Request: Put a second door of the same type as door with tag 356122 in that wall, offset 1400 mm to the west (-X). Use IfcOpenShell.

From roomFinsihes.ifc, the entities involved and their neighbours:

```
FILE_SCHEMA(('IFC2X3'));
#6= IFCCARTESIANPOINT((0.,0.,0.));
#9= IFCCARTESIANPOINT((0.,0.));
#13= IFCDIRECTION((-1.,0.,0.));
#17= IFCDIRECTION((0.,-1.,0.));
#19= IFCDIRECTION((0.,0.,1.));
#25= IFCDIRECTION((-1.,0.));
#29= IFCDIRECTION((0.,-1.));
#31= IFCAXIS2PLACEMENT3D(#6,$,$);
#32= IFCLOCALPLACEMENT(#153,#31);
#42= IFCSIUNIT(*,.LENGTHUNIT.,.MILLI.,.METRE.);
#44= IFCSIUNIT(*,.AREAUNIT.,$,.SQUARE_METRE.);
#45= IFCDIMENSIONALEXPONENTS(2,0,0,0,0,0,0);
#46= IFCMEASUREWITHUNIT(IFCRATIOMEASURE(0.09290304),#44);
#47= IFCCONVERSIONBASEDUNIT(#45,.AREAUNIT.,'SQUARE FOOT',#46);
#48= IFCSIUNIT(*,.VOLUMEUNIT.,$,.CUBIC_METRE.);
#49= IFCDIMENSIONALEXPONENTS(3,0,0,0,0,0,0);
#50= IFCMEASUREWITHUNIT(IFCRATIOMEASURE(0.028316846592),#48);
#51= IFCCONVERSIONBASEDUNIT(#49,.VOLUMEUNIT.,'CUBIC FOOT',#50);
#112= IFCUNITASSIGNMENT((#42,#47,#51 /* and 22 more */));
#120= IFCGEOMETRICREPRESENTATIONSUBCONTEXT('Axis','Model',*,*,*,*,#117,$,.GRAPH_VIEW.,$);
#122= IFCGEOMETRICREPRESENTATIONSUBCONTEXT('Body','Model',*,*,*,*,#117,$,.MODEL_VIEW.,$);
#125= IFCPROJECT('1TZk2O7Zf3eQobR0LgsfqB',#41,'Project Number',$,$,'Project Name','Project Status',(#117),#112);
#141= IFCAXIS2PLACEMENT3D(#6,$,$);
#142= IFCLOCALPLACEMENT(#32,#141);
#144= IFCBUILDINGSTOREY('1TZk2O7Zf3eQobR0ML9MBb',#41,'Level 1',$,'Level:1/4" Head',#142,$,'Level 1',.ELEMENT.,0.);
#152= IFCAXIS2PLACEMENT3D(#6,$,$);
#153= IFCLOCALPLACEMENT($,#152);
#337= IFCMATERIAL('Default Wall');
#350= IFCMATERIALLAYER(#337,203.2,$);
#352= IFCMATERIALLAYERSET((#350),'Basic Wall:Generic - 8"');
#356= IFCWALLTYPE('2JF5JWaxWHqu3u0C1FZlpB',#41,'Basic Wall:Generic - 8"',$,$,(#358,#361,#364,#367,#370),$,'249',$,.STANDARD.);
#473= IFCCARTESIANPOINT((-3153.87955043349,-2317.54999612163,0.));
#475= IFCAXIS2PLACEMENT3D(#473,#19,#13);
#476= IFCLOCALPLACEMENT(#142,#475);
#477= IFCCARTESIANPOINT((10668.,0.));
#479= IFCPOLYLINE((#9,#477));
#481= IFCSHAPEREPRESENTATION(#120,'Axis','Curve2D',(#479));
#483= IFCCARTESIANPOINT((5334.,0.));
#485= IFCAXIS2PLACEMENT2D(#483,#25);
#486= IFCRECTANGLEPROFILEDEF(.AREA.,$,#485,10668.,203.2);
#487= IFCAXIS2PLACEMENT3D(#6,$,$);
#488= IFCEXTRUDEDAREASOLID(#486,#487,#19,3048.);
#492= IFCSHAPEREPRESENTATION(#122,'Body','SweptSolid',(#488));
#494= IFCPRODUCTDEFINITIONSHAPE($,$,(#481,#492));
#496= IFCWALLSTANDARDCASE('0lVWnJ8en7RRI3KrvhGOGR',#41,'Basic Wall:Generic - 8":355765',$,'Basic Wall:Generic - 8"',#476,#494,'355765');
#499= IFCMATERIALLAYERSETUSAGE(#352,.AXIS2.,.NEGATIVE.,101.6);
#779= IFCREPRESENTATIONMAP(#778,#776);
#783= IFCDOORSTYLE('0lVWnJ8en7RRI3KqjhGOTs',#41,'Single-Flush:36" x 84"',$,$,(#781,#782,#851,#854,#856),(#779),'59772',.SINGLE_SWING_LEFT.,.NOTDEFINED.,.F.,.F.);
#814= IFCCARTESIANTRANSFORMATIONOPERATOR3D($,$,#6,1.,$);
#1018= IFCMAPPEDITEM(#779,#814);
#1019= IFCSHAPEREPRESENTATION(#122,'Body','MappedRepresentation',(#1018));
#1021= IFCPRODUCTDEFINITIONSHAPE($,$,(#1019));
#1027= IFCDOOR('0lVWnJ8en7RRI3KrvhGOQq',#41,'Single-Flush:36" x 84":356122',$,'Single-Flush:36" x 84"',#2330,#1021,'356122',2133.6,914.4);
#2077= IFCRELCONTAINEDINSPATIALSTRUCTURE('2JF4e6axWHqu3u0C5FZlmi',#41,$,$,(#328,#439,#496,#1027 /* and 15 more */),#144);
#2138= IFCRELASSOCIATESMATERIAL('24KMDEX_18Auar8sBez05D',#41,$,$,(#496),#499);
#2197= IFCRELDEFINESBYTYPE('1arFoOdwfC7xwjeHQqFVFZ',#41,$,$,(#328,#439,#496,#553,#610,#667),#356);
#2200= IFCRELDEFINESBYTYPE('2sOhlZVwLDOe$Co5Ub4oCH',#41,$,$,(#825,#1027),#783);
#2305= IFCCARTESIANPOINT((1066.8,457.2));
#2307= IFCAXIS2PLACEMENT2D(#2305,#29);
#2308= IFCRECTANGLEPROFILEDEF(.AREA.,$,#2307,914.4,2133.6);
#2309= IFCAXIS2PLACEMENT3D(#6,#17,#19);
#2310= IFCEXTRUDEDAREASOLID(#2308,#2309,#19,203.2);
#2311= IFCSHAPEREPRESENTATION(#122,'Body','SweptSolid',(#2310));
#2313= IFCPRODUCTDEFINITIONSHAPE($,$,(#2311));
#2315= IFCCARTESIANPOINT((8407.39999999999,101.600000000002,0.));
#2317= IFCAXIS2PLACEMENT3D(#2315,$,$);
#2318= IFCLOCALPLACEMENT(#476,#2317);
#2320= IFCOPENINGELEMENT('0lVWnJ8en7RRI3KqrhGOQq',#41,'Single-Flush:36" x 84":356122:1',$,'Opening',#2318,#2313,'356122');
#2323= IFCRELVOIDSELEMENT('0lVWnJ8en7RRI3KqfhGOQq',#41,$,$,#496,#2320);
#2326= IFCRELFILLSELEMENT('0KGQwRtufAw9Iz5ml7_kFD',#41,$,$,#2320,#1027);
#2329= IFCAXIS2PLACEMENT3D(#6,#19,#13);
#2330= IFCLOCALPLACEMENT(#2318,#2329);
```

```python
import ifcopenshell
import ifcopenshell.api.feature
import ifcopenshell.api.geometry
import ifcopenshell.api.root
import ifcopenshell.geom
import ifcopenshell.util.element
import ifcopenshell.util.placement
import ifcopenshell.util.shape
import ifcopenshell.util.unit

model = ifcopenshell.open("roomFinsihes.ifc")
unit_scale = ifcopenshell.util.unit.calculate_unit_scale(model)
settings = ifcopenshell.geom.settings()


def volume(element):
    """Net volume in cubic metres, openings subtracted."""
    shape = ifcopenshell.geom.create_shape(settings, element)
    return ifcopenshell.util.shape.get_volume(shape.geometry)


def reuse_history(source, copy):
    """copy_class also copies each property set's owner history, people and application; keep the originals."""
    for rel in copy.IsDefinedBy:
        if rel.is_a("IfcRelDefinesByProperties") and (history := rel.RelatingPropertyDefinition.OwnerHistory):
            rel.RelatingPropertyDefinition.OwnerHistory = source.OwnerHistory
            ifcopenshell.util.element.remove_deep2(model, history)


door = model.by_guid("0lVWnJ8en7RRI3KrvhGOQq")
opening = door.FillsVoids[0].RelatingOpeningElement
wall = opening.VoidsElements[0].RelatingBuildingElement
before = volume(wall)
shift = ifcopenshell.util.placement.get_local_placement(wall.ObjectPlacement)[:3, 0] * 1.4 / unit_scale

# copy_class copies the void relationship, type, container and properties, but no geometry.
new_opening = ifcopenshell.api.root.copy_class(model, product=opening)
new_opening.Representation = ifcopenshell.util.element.copy_deep(
    model, opening.Representation, exclude=["IfcGeometricRepresentationContext", "IfcRepresentationMap"]
)
new_opening.Name = 'Single-Flush:36" x 84"'
new_opening.Tag = None
new_door = ifcopenshell.api.root.copy_class(model, product=door)
new_door.Representation = ifcopenshell.util.element.copy_deep(
    model, door.Representation, exclude=["IfcGeometricRepresentationContext", "IfcRepresentationMap"]
)
new_door.Name = 'Single-Flush:36" x 84"'
new_door.Tag = None
reuse_history(door, new_door)
fills = ifcopenshell.api.feature.add_filling(model, opening=new_opening, element=new_door)
fills.OwnerHistory = new_door.OwnerHistory  # required in IFC2X3

for old, new in ((opening, new_opening), (door, new_door)):
    matrix = ifcopenshell.util.placement.get_local_placement(old.ObjectPlacement)
    matrix[:3, 3] += shift
    ifcopenshell.api.geometry.edit_object_placement(model, product=new, matrix=matrix, is_si=False)

after = volume(wall)

print(f"wall volume {before:.3f} -> {after:.3f} m3")

model.write("roomFinsihes_rev.ifc")
```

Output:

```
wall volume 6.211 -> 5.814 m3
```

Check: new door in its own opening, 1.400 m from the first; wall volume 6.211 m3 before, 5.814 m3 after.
